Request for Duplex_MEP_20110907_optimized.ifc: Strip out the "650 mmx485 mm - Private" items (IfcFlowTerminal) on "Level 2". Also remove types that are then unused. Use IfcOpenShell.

First a look at what the model holds.

```python
import ifcopenshell
import ifcopenshell.util.element

model = ifcopenshell.open("Duplex_MEP_20110907_optimized.ifc")
print(model.schema)
storey = next(s for s in model.by_type("IfcBuildingStorey") if s.Name == "Level 2")
terminals = [e for e in ifcopenshell.util.element.get_decomposition(storey) if e.is_a("IfcFlowTerminal")]
seen = {}
for e in terminals:
    element_type = ifcopenshell.util.element.get_type(e)
    name = element_type.Name if element_type not in (None, e) else None
    seen[name] = seen.get(name, 0) + 1
for name, count in sorted(seen.items(), key=str):
    print(count, "x", name)
```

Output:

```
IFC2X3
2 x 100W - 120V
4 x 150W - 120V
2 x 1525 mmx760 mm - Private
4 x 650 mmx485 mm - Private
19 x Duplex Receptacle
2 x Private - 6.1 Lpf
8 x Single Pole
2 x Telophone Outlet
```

```python
import ifcopenshell
import ifcopenshell.api.root
import ifcopenshell.util.element

model = ifcopenshell.open("Duplex_MEP_20110907_optimized.ifc")

storey = next(s for s in model.by_type("IfcBuildingStorey") if s.Name == "Level 2")
terminals = [e for e in ifcopenshell.util.element.get_decomposition(storey) if e.is_a("IfcFlowTerminal")]
targets = [e for e in terminals if (t := ifcopenshell.util.element.get_type(e)) not in (None, e) and t.Name == "650 mmx485 mm - Private"]
types = {ifcopenshell.util.element.get_type(e) for e in targets} - {None, *targets}

for e in targets:
    ifcopenshell.api.root.remove_product(model, product=e)
print(len(targets), "removed")

unused = [t for t in types if not ifcopenshell.util.element.get_types(t)]
for t in unused:
    ifcopenshell.api.root.remove_product(model, product=t)
print(len(unused), "unused types removed")

model.write("Duplex_MEP_20110907_optimized_updated.ifc")
```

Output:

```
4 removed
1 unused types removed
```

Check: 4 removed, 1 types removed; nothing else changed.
